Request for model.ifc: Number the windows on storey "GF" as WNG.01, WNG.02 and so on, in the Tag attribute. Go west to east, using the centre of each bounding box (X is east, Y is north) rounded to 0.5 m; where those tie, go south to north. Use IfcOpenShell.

First a look at what the model holds.

```python
import ifcopenshell
import ifcopenshell.util.element
import ifcopenshell.util.placement

model = ifcopenshell.open("model.ifc")
print(model.schema)
storey = next(s for s in model.by_type("IfcBuildingStorey") if s.Name == "GF")
windows = [e for e in ifcopenshell.util.element.get_decomposition(storey) if e.is_a("IfcWindow")]
for e in sorted(windows, key=lambda e: e.id()):
    origin = ifcopenshell.util.placement.get_local_placement(e.ObjectPlacement)[:3, 3]
    print(e.id(), e.Tag, e.Name, origin.round(2) + 0.0, sep=" | ")
```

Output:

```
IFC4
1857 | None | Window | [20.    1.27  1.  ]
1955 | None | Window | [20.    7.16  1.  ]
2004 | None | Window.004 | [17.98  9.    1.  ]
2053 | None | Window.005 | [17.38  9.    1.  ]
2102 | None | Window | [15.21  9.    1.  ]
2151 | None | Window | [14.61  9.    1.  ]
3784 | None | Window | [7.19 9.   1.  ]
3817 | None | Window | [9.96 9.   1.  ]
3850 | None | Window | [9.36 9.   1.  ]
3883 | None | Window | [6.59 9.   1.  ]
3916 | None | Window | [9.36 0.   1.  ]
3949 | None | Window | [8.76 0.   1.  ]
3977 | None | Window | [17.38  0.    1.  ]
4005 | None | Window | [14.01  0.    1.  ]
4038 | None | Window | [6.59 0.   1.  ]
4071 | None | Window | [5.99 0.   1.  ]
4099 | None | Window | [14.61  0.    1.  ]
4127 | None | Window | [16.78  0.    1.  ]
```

```python
import ifcopenshell
import ifcopenshell.geom
import ifcopenshell.util.element
import ifcopenshell.util.shape

model = ifcopenshell.open("model.ifc")
settings = ifcopenshell.geom.settings()
settings.set("use-world-coords", True)


def centre(element):
    shape = ifcopenshell.geom.create_shape(settings, element)
    return ifcopenshell.util.shape.get_bbox_centroid(shape.geometry)


storey = next(s for s in model.by_type("IfcBuildingStorey") if s.Name == "GF")
windows = [e for e in ifcopenshell.util.element.get_decomposition(storey) if e.is_a("IfcWindow")]

# Insertion points can sit at a corner or the storey origin, so sort by the geometry (in metres).
centres = {e: centre(e) for e in windows}
windows.sort(key=lambda e: (round(centres[e][0] / 0.5), centres[e][1]))

for i, e in enumerate(windows, start=1):
    number = f"WNG.{i:02d}"
    e.Tag = number
    print(e.id(), number)

model.write("model_updated.ifc")
```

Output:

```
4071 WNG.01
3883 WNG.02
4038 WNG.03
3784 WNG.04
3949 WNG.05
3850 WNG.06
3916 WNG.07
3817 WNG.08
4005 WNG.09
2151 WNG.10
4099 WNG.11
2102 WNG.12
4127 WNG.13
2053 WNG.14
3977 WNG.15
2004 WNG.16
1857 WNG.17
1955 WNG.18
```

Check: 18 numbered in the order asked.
